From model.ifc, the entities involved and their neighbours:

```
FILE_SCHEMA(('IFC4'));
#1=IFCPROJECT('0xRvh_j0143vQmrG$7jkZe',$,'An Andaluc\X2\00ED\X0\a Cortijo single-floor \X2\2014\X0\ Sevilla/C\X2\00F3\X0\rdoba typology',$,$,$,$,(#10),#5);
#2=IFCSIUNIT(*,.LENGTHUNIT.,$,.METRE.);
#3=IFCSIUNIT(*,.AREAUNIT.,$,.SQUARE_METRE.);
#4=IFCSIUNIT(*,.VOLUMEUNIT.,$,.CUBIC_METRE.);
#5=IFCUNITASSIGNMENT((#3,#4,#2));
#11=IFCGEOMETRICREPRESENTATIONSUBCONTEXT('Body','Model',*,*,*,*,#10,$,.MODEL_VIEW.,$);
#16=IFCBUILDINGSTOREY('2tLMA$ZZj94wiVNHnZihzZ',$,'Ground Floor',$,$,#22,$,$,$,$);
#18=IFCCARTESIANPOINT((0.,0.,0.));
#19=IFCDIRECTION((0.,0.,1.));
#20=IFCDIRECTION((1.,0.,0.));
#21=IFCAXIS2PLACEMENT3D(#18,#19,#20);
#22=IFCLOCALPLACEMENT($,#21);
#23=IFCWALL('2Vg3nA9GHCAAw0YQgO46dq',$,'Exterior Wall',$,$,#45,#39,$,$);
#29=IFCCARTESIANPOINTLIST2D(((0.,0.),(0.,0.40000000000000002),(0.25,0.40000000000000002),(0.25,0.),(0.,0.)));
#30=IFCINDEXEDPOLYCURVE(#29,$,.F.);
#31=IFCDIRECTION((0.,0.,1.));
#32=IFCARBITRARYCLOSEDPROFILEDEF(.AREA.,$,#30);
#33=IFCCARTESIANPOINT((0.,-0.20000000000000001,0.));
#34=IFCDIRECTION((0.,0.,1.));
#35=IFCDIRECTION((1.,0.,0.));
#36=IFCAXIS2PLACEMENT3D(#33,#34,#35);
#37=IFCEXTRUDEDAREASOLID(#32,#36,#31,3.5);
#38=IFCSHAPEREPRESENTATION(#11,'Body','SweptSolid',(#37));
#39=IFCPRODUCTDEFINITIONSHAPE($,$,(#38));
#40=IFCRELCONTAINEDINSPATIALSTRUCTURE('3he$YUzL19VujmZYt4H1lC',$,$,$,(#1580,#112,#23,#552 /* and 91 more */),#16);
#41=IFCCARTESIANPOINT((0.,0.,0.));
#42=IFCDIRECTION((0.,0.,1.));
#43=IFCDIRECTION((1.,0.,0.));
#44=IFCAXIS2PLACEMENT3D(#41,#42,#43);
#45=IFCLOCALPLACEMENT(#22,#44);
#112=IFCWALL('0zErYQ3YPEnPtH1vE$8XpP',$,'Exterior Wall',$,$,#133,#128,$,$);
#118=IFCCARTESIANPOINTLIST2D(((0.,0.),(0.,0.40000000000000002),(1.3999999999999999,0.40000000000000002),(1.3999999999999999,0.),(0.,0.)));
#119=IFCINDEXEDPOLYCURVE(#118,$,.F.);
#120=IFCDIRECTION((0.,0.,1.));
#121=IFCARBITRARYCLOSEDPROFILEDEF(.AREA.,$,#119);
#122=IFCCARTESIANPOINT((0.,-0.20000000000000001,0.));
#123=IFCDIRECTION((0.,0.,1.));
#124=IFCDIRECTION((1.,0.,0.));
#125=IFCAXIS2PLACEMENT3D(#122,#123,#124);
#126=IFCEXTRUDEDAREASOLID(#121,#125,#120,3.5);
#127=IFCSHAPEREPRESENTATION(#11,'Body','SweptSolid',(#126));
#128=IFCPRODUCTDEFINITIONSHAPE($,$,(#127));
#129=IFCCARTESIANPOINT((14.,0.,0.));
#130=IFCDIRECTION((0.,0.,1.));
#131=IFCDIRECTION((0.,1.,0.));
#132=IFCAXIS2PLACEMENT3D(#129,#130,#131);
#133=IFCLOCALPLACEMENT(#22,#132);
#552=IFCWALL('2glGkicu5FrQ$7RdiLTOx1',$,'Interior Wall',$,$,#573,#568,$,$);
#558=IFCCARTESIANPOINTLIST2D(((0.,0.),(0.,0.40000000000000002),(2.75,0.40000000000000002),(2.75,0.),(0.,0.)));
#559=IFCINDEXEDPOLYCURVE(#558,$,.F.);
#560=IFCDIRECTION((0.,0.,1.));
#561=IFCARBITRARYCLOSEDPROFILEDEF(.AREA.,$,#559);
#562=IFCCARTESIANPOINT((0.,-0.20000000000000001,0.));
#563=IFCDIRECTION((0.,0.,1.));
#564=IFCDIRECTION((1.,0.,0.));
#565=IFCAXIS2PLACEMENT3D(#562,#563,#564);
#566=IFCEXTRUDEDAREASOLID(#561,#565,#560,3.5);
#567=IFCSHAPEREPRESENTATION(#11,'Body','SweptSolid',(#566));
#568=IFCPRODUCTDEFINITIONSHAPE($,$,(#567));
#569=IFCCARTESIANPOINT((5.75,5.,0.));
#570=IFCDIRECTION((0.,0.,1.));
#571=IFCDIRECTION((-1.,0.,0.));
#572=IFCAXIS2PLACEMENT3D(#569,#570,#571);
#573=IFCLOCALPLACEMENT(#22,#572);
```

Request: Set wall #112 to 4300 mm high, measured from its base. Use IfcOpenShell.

```python
import ifcopenshell
import ifcopenshell.geom
import ifcopenshell.util.representation
import ifcopenshell.util.shape
import ifcopenshell.util.unit

model = ifcopenshell.open("model.ifc")
unit_scale = ifcopenshell.util.unit.calculate_unit_scale(model)
settings = ifcopenshell.geom.settings()


def volume(element):
    """Net volume in cubic metres, openings subtracted."""
    shape = ifcopenshell.geom.create_shape(settings, element)
    return ifcopenshell.util.shape.get_volume(shape.geometry)


wall = model.by_id(112)
before = volume(wall)

body = ifcopenshell.util.representation.get_representation(wall, "Model", "Body")
solid = body.Items[0]
old_height = solid.Depth
solid.Depth = 4.3 / unit_scale
after = volume(wall)

print(f"height {old_height:g} -> {solid.Depth:g}, volume {before:.3f} -> {after:.3f} m3")

model.write("model_edited.ifc")
```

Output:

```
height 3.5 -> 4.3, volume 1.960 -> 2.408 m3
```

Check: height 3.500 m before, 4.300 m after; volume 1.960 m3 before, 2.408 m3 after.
